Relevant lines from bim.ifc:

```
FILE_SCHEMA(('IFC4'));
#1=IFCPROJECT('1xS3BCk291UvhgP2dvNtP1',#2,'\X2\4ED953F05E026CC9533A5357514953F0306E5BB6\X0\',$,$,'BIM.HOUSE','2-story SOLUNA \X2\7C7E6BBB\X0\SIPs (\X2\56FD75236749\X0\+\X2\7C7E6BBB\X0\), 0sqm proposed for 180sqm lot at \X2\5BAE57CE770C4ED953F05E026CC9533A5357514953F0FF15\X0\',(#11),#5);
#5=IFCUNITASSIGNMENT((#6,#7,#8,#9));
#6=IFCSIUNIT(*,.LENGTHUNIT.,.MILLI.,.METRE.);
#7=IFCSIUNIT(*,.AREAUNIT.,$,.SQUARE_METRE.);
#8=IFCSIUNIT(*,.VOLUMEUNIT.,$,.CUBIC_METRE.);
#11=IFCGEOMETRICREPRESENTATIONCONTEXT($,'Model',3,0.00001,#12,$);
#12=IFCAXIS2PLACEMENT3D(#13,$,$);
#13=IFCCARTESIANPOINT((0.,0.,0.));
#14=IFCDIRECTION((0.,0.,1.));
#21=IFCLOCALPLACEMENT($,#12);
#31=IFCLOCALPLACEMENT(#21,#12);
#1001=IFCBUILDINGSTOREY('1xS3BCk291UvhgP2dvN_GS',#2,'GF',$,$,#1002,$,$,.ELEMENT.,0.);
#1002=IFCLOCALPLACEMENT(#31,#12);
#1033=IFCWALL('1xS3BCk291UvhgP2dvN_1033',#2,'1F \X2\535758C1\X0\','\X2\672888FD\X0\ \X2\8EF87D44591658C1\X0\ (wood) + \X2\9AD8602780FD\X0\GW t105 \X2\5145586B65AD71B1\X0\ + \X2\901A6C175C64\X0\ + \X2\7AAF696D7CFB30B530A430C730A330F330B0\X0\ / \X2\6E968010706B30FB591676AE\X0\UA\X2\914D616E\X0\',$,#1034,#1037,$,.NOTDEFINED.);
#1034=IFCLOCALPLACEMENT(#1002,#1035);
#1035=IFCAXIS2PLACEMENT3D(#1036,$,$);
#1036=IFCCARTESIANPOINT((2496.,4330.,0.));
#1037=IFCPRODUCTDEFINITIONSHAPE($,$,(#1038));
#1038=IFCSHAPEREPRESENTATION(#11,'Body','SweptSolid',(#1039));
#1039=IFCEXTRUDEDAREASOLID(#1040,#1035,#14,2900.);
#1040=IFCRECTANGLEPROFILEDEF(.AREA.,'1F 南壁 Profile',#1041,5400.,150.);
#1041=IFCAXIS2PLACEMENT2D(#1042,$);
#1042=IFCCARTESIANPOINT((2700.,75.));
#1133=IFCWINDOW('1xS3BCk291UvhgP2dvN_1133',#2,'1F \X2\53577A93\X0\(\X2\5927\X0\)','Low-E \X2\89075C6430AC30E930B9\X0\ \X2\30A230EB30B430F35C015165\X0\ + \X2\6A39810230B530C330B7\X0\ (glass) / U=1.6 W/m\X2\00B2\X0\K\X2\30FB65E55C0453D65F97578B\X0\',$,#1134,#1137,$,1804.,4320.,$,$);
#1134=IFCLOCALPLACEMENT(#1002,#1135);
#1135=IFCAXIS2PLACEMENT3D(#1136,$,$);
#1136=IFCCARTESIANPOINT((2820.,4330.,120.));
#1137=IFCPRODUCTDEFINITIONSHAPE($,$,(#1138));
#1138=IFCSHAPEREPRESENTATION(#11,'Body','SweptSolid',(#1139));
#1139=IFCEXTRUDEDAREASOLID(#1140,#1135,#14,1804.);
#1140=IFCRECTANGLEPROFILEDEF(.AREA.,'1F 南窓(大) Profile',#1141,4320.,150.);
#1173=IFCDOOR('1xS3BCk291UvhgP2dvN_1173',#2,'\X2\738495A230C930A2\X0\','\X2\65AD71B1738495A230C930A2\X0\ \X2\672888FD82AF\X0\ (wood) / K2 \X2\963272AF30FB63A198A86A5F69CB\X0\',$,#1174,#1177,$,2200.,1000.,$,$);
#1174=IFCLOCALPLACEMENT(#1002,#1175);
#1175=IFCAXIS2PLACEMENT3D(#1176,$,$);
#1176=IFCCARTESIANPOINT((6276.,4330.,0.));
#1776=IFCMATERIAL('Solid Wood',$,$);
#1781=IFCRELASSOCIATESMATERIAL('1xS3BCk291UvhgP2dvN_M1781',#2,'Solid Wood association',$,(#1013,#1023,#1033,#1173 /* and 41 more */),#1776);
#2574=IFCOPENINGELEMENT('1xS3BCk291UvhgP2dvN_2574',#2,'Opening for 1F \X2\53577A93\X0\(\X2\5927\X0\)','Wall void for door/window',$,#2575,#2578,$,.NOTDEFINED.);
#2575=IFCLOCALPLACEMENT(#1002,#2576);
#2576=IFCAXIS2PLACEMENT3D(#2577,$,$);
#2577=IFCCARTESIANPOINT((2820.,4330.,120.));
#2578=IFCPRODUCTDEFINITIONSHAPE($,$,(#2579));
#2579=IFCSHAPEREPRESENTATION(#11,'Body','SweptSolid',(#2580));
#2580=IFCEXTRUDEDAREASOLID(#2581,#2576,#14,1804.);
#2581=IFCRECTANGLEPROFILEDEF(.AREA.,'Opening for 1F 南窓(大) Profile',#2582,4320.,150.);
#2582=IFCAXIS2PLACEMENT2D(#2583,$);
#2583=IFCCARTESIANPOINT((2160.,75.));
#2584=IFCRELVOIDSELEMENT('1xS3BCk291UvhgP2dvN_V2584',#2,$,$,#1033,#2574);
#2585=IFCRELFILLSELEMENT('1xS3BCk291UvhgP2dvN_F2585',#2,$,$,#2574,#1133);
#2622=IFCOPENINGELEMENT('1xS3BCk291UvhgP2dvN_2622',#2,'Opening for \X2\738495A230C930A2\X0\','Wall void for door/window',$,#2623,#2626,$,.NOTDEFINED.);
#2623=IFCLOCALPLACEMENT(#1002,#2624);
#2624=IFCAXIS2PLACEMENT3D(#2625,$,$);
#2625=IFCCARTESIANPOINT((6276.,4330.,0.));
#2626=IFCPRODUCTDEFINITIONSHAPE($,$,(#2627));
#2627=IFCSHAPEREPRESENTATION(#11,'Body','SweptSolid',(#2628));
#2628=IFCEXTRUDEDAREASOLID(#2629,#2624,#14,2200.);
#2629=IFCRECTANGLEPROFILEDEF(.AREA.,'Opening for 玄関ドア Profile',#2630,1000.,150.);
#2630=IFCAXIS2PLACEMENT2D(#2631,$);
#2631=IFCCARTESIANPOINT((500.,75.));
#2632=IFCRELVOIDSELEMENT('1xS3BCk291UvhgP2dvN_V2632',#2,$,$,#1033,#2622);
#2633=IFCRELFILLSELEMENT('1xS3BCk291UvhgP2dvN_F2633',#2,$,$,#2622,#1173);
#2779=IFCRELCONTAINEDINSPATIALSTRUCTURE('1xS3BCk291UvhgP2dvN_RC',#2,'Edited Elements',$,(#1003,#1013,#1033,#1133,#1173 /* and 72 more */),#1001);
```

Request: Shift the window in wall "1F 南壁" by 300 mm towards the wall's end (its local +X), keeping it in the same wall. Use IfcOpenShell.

```python
import ifcopenshell
import ifcopenshell.api.geometry
import ifcopenshell.util.placement

model = ifcopenshell.open("bim.ifc")

window = model.by_id(1133)
opening = window.FillsVoids[0].RelatingOpeningElement
wall = opening.VoidsElements[0].RelatingBuildingElement

wall_matrix = ifcopenshell.util.placement.get_local_placement(wall.ObjectPlacement)
shift = wall_matrix[:3, 0] * 300.0
before = ifcopenshell.util.placement.get_local_placement(window.ObjectPlacement)[:3, 3].copy()

# The window is not placed relative to its opening, so move both.
for product in (opening, window):
    matrix = ifcopenshell.util.placement.get_local_placement(product.ObjectPlacement)
    matrix[:3, 3] += shift
    ifcopenshell.api.geometry.edit_object_placement(model, product=product, matrix=matrix, is_si=False)

after = ifcopenshell.util.placement.get_local_placement(window.ObjectPlacement)[:3, 3]
print("window moved by", (after - before).round(3) + 0.0)

model.write("bim_rev.ifc")
```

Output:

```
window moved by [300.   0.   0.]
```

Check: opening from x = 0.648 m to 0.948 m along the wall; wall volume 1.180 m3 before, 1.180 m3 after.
